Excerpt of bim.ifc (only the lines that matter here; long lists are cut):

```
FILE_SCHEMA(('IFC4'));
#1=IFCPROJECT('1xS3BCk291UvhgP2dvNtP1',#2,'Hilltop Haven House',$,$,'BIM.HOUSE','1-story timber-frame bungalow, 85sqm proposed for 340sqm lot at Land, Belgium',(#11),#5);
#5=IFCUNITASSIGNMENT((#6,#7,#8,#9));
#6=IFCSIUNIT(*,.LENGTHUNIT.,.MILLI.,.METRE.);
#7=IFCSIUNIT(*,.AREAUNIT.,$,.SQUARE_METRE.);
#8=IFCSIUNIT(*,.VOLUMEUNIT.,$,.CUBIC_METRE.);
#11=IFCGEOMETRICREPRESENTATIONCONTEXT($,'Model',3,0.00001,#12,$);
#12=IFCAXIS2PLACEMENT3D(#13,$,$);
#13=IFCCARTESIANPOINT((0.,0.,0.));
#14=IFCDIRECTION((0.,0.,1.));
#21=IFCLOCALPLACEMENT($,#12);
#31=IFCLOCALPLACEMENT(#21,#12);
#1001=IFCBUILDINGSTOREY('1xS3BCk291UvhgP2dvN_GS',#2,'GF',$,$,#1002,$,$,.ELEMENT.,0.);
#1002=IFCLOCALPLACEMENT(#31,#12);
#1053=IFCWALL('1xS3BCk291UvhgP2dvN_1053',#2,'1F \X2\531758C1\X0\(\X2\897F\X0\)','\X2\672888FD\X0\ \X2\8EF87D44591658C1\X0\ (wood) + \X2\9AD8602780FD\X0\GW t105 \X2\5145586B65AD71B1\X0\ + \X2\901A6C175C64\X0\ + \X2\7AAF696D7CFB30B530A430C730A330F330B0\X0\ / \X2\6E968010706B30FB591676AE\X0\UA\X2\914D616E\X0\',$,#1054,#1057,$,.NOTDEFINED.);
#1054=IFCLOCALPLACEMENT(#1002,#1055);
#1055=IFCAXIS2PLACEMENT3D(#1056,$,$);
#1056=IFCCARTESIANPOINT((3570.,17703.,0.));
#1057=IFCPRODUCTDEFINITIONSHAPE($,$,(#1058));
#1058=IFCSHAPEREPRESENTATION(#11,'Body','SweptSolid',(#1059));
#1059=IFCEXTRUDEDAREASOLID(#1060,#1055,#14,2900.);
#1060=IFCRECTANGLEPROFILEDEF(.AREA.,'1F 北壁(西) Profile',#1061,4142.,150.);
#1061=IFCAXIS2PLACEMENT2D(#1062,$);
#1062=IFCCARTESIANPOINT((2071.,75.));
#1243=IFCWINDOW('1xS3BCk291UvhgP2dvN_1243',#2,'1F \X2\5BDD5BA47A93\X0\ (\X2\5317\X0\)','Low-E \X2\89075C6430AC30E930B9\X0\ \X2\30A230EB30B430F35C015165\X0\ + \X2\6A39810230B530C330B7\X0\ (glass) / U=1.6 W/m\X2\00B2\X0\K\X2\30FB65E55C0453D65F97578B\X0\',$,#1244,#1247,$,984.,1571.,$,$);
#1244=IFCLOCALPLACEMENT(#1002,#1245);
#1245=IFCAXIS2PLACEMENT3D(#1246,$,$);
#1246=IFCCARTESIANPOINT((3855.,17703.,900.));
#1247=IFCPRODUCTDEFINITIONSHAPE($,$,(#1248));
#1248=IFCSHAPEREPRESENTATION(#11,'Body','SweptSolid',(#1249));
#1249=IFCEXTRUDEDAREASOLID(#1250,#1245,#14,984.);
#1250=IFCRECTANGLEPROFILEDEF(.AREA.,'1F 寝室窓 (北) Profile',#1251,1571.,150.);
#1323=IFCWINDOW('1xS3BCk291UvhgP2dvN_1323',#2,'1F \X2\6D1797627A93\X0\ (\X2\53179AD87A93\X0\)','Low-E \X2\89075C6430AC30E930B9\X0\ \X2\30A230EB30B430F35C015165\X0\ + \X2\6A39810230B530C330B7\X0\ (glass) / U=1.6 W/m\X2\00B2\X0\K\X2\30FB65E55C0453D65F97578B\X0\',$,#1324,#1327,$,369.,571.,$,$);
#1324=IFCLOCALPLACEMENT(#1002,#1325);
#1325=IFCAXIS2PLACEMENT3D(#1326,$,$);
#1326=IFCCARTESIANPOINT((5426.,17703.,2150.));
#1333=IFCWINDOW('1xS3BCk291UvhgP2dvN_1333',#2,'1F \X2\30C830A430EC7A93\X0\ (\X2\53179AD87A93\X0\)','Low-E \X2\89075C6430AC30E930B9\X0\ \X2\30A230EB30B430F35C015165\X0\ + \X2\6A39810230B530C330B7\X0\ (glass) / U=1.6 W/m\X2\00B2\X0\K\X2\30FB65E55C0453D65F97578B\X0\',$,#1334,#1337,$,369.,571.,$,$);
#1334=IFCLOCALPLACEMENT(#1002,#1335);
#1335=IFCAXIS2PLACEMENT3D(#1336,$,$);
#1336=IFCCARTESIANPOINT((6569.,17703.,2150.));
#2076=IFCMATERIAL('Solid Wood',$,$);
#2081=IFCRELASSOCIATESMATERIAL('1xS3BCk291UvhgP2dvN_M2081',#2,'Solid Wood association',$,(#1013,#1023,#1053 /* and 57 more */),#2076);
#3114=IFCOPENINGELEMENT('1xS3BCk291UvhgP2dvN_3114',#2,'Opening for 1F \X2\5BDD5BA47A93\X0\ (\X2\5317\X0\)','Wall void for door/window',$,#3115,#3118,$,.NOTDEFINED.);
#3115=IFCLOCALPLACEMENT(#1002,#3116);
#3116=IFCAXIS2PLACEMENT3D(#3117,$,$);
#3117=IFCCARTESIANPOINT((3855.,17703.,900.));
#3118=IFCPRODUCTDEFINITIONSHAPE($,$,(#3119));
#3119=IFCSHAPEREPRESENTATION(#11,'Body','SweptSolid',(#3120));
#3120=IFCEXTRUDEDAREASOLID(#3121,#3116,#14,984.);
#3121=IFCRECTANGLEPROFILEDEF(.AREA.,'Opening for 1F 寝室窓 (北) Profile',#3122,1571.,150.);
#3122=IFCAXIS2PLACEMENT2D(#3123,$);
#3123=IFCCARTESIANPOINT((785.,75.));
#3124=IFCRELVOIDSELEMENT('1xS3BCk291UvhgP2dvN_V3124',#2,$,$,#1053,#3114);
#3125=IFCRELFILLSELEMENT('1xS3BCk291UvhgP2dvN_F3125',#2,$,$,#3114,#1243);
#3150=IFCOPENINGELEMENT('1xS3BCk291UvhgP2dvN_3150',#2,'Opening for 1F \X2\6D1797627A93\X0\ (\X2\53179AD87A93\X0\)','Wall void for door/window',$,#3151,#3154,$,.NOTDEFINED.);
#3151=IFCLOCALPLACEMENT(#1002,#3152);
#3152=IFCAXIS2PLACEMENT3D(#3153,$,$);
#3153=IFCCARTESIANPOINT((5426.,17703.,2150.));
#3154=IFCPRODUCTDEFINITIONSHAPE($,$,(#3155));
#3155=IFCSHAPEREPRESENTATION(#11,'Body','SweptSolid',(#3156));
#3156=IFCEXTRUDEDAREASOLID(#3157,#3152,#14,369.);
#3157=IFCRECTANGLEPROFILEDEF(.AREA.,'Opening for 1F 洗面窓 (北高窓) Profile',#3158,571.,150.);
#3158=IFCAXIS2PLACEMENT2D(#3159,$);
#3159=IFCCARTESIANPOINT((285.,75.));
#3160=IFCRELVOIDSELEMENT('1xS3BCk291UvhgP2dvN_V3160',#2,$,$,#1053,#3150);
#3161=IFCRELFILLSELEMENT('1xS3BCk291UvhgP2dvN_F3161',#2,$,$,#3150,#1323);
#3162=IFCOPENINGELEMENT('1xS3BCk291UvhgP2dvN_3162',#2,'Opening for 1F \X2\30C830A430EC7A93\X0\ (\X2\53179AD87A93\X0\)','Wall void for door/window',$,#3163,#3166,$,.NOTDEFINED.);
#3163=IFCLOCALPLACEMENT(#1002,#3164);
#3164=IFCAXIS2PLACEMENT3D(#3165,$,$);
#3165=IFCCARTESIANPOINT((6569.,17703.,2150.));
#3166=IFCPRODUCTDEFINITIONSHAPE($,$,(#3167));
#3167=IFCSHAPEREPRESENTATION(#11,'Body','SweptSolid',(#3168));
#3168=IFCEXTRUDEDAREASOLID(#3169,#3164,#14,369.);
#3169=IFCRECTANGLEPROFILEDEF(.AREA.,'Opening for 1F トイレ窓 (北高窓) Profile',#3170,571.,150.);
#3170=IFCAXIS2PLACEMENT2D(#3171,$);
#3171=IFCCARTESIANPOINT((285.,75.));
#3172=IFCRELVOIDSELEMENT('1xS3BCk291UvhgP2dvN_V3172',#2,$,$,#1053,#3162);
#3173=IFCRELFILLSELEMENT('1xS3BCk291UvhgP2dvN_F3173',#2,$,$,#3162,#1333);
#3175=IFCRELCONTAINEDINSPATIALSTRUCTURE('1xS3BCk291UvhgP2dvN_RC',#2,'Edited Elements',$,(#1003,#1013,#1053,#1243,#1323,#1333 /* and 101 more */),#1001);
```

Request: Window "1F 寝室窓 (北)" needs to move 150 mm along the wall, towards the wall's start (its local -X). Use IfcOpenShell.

```python
import ifcopenshell
import ifcopenshell.api.geometry
import ifcopenshell.util.placement

model = ifcopenshell.open("bim.ifc")

window = model.by_guid("1xS3BCk291UvhgP2dvN_1243")
opening = window.FillsVoids[0].RelatingOpeningElement
wall = opening.VoidsElements[0].RelatingBuildingElement

wall_matrix = ifcopenshell.util.placement.get_local_placement(wall.ObjectPlacement)
shift = wall_matrix[:3, 0] * -150.0
before = ifcopenshell.util.placement.get_local_placement(window.ObjectPlacement)[:3, 3].copy()

# The window is not placed relative to its opening, so move both.
for product in (opening, window):
    matrix = ifcopenshell.util.placement.get_local_placement(product.ObjectPlacement)
    matrix[:3, 3] += shift
    ifcopenshell.api.geometry.edit_object_placement(model, product=product, matrix=matrix, is_si=False)

after = ifcopenshell.util.placement.get_local_placement(window.ObjectPlacement)[:3, 3]
print("window moved by", (after - before).round(3) + 0.0)

model.write("bim_edited.ifc")
```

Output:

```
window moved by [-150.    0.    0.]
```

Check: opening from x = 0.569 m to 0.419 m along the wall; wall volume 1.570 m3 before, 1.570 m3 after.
